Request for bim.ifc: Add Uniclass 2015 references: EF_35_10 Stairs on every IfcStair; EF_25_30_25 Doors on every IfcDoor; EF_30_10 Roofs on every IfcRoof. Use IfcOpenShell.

First a look at what the model holds.

```python
import ifcopenshell

model = ifcopenshell.open("bim.ifc")
print(model.schema)
print("classifications:", [c.Name for c in model.by_type("IfcClassification")])
for ifc_class in ("IfcDoor", "IfcRoof", "IfcStair", "IfcWall", "IfcWindow"):
    print(ifc_class, len(model.by_type(ifc_class)))
```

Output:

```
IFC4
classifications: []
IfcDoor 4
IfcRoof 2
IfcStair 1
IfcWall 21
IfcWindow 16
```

```python
import ifcopenshell
import ifcopenshell.api.classification

model = ifcopenshell.open("bim.ifc")

system = ifcopenshell.api.classification.add_classification(model, classification="Uniclass 2015")

codes = {
    "IfcStair": ("EF_35_10", "Stairs"),
    "IfcDoor": ("EF_25_30_25", "Doors"),
    "IfcRoof": ("EF_30_10", "Roofs"),
}
for ifc_class, (code, name) in codes.items():
    products = model.by_type(ifc_class)
    ifcopenshell.api.classification.add_reference(
        model, products=products, classification=system, identification=code, name=name
    )
    print(code, len(products))

model.write("bim_edited.ifc")
```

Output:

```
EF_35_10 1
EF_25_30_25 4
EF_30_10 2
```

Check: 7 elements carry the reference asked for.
